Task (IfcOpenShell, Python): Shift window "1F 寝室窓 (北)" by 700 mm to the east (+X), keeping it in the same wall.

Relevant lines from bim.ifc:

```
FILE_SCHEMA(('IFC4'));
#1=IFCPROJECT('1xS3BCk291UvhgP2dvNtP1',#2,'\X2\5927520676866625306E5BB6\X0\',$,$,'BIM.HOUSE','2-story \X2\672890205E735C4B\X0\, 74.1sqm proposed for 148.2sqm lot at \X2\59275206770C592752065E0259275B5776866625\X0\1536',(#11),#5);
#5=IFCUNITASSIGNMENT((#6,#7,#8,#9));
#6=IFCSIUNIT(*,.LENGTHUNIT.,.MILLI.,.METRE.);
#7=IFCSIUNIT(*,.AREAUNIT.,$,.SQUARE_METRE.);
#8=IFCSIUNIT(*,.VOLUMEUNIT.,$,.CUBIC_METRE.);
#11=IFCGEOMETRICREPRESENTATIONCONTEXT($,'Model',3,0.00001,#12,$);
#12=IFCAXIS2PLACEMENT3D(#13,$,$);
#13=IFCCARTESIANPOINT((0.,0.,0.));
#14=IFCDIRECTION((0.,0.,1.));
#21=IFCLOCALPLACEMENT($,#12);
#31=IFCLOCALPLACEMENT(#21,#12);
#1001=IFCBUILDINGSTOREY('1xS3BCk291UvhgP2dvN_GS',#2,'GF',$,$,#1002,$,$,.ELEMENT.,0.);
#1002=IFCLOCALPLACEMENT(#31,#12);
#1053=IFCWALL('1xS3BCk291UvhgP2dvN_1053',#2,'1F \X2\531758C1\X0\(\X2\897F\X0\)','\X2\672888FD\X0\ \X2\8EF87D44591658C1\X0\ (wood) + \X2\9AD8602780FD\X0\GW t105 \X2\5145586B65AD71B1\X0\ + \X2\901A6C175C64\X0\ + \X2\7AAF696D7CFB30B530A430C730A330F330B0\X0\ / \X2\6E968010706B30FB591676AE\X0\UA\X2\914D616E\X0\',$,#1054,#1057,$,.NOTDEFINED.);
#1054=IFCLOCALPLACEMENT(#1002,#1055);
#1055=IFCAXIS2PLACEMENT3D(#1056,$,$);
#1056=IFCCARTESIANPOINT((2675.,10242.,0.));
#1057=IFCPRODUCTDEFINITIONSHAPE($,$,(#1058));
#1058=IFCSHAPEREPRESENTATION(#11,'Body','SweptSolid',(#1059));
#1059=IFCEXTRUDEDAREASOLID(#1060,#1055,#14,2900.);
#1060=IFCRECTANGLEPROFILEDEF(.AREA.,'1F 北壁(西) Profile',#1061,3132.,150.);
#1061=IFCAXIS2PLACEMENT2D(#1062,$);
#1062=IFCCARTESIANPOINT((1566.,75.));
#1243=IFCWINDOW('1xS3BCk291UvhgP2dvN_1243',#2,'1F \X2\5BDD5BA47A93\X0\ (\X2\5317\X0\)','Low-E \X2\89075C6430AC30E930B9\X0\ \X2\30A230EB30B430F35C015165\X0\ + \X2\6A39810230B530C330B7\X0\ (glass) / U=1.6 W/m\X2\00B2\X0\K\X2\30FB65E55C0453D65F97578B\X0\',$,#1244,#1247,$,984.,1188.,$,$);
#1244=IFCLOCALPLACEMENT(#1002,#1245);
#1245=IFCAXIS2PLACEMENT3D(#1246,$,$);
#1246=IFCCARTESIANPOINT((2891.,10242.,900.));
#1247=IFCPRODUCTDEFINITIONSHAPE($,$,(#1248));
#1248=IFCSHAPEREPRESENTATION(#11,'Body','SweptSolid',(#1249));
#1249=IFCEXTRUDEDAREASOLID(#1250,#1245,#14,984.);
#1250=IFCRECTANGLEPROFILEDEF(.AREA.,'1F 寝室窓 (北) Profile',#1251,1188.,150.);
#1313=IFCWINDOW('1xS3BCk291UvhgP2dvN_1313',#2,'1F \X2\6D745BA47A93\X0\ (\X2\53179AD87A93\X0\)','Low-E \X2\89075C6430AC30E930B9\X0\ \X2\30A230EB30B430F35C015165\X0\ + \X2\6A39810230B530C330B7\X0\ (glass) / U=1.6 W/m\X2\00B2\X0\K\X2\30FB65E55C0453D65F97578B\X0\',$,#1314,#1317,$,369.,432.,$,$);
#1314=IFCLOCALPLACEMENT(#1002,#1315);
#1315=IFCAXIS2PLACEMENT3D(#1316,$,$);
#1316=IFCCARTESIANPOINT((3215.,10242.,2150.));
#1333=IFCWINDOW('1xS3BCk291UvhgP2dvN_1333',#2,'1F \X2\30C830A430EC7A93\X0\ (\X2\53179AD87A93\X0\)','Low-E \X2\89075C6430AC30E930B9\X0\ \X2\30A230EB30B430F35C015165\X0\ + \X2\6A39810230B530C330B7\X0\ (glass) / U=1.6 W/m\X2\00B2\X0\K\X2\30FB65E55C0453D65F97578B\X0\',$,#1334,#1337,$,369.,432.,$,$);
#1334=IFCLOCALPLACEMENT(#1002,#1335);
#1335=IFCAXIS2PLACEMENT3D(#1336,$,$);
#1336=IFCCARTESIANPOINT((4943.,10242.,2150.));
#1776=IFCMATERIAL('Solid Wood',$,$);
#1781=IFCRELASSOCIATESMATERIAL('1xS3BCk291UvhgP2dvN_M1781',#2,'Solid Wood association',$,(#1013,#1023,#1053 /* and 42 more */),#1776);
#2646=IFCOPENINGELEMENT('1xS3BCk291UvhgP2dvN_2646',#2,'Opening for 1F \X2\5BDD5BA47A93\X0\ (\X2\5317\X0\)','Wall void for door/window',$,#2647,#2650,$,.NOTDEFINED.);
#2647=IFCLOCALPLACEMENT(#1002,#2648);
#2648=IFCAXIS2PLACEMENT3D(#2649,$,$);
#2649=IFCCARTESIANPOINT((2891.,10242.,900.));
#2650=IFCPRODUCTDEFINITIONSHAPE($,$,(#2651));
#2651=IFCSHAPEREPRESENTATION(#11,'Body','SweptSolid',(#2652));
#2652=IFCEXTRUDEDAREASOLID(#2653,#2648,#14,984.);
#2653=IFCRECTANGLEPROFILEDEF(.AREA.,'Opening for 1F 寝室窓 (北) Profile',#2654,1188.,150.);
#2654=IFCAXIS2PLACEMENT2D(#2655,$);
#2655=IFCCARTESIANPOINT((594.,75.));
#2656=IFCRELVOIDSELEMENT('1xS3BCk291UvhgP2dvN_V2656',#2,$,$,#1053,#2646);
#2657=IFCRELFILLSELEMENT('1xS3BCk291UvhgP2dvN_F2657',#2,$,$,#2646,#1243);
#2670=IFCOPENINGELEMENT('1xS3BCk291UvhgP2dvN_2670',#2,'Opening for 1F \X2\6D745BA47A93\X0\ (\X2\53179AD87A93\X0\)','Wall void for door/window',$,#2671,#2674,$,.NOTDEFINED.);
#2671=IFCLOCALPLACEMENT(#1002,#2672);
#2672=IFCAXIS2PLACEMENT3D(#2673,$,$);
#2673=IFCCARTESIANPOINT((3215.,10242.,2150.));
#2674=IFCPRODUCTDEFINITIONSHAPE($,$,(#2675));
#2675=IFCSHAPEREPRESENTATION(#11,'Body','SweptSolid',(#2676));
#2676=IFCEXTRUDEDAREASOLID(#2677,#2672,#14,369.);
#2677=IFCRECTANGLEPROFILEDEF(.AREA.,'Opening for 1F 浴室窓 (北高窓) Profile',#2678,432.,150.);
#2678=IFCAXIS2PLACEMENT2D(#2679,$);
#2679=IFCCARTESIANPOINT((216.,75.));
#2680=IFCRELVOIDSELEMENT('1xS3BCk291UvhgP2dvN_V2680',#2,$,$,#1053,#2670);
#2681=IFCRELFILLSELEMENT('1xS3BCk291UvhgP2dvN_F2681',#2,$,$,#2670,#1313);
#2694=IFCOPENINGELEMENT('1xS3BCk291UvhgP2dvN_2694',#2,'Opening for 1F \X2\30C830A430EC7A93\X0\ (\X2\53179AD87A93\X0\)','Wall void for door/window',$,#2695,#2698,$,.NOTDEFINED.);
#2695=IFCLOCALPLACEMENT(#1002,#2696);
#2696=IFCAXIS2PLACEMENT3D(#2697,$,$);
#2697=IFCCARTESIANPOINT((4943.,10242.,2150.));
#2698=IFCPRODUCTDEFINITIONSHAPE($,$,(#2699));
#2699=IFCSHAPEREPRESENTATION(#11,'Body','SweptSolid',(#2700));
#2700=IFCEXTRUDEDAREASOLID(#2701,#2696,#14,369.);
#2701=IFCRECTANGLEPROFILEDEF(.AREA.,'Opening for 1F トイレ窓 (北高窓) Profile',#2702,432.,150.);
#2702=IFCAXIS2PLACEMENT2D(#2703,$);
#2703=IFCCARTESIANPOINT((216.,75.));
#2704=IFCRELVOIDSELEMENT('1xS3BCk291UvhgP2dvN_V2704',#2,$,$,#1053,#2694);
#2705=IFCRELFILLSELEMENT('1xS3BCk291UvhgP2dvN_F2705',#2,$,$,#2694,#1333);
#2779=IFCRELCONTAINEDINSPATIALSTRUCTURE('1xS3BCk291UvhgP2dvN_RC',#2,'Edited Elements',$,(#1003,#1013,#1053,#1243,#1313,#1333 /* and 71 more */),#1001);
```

```python
import ifcopenshell
import ifcopenshell.api.geometry
import ifcopenshell.util.placement

model = ifcopenshell.open("bim.ifc")

window = model.by_guid("1xS3BCk291UvhgP2dvN_1243")
opening = window.FillsVoids[0].RelatingOpeningElement
wall = opening.VoidsElements[0].RelatingBuildingElement

wall_matrix = ifcopenshell.util.placement.get_local_placement(wall.ObjectPlacement)
shift = wall_matrix[:3, 0] * 700.0
before = ifcopenshell.util.placement.get_local_placement(window.ObjectPlacement)[:3, 3].copy()

# The window is not placed relative to its opening, so move both.
for product in (opening, window):
    matrix = ifcopenshell.util.placement.get_local_placement(product.ObjectPlacement)
    matrix[:3, 3] += shift
    ifcopenshell.api.geometry.edit_object_placement(model, product=product, matrix=matrix, is_si=False)

after = ifcopenshell.util.placement.get_local_placement(window.ObjectPlacement)[:3, 3]
print("window moved by", (after - before).round(3) + 0.0)

model.write("bim_rev.ifc")
```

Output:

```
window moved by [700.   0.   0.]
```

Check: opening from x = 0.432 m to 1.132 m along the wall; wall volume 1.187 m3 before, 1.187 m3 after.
